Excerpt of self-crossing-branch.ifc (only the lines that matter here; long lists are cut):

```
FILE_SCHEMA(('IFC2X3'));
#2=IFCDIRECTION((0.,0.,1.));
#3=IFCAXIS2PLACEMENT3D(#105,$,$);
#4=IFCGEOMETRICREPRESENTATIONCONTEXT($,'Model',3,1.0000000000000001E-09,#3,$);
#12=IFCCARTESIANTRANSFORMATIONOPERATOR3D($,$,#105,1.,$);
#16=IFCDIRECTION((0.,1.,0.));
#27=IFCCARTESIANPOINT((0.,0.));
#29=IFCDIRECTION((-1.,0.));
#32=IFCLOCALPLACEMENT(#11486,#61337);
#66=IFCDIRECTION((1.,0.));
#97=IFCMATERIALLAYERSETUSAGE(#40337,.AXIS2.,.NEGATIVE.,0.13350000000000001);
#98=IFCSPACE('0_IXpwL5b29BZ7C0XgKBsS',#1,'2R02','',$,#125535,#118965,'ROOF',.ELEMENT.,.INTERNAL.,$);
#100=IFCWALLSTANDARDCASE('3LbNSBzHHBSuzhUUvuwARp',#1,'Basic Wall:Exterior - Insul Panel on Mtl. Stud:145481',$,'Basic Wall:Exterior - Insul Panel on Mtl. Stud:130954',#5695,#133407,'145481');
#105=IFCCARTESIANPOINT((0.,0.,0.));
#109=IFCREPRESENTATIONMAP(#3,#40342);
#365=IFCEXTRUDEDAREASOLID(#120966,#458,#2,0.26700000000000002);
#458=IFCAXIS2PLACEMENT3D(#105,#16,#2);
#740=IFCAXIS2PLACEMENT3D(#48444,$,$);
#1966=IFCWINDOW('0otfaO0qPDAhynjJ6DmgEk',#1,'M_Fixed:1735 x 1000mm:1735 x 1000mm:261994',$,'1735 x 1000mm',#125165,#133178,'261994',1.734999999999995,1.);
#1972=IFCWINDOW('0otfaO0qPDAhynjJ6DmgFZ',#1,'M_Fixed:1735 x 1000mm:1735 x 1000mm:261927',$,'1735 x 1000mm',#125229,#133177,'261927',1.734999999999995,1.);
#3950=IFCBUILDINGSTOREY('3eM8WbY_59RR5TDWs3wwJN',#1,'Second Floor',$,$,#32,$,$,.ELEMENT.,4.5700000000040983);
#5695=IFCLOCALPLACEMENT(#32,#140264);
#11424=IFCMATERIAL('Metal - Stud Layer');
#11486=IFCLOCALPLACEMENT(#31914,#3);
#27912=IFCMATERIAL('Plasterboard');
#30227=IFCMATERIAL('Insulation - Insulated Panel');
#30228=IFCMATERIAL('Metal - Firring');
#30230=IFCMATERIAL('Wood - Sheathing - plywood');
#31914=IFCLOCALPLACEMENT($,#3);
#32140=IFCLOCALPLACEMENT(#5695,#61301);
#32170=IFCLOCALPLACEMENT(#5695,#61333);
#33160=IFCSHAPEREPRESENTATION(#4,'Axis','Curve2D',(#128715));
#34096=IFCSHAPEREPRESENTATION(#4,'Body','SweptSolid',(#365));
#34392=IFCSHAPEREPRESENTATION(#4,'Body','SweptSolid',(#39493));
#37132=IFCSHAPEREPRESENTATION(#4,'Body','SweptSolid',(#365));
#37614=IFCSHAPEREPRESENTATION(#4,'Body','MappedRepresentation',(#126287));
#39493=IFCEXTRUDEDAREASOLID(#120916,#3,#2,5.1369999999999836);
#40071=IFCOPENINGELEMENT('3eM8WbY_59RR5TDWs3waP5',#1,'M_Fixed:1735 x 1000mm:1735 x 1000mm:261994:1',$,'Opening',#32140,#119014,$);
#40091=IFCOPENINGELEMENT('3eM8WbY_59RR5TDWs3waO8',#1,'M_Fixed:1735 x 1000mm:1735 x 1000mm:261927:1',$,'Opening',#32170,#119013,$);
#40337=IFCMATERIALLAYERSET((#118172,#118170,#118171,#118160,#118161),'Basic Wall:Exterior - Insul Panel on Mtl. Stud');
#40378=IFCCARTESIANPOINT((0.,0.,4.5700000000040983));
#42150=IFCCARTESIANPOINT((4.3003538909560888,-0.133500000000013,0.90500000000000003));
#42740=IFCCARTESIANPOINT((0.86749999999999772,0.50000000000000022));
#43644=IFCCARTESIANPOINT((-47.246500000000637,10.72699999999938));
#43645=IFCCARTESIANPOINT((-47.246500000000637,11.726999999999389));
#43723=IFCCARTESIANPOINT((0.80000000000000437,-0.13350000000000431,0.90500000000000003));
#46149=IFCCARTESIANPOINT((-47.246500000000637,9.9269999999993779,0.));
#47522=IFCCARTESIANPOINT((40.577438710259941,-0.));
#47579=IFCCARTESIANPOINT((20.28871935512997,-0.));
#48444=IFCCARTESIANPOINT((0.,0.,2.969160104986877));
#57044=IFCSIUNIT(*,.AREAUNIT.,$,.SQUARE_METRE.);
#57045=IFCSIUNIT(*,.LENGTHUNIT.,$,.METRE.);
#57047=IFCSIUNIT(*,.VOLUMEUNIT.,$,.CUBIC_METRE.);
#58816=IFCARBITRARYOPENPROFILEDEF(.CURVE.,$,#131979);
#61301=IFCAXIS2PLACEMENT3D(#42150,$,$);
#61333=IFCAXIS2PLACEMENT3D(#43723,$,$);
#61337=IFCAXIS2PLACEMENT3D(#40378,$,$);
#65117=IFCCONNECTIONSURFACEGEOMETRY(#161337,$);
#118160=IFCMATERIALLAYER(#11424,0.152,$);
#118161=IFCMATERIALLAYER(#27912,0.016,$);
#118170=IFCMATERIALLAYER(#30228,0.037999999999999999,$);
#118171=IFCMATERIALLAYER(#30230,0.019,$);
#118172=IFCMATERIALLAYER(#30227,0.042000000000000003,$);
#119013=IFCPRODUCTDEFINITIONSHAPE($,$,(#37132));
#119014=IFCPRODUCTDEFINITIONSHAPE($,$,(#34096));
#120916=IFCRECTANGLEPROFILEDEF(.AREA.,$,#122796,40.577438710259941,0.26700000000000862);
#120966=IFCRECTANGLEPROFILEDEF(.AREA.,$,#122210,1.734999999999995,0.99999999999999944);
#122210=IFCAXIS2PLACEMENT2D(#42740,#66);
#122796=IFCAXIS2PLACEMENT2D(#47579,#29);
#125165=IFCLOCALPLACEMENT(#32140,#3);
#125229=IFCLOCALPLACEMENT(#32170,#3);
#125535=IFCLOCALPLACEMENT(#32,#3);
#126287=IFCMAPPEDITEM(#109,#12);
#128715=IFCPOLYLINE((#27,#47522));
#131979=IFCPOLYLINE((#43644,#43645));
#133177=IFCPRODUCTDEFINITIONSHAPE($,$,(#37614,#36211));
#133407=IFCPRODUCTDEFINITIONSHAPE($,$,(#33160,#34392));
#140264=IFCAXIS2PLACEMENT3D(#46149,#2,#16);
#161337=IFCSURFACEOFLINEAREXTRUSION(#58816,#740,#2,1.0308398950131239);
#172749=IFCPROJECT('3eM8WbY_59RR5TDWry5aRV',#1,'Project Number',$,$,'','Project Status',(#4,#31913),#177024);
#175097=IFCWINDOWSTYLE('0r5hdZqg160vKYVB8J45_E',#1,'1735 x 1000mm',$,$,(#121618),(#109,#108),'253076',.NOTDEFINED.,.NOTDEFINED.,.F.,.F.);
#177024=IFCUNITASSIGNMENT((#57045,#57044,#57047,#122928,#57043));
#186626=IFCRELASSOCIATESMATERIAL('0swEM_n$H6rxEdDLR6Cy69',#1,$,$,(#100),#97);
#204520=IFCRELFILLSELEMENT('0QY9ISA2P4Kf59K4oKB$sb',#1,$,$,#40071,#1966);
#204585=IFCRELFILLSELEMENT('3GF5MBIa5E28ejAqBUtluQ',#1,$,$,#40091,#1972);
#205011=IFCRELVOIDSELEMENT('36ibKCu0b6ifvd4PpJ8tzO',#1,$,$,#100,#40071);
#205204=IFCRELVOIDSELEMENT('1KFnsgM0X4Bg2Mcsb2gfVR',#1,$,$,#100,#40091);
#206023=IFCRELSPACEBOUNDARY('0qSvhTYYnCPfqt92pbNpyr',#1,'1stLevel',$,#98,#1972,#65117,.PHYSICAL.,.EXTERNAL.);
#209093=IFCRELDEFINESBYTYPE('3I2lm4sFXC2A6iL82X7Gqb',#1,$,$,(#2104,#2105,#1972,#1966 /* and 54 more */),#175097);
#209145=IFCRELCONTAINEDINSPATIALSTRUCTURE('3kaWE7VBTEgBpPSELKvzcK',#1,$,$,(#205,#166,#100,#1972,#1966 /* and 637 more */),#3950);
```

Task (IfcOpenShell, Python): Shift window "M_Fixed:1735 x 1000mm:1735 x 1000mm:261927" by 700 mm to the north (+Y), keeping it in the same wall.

```python
import numpy as np
import ifcopenshell
import ifcopenshell.api.geometry
import ifcopenshell.util.placement
import ifcopenshell.util.unit

model = ifcopenshell.open("self-crossing-branch.ifc")
unit_scale = ifcopenshell.util.unit.calculate_unit_scale(model)

window = model.by_guid("0otfaO0qPDAhynjJ6DmgFZ")
opening = window.FillsVoids[0].RelatingOpeningElement
wall = opening.VoidsElements[0].RelatingBuildingElement

wall_matrix = ifcopenshell.util.placement.get_local_placement(wall.ObjectPlacement)
shift = wall_matrix[:3, 0] * 0.7 / unit_scale
before = ifcopenshell.util.placement.get_local_placement(window.ObjectPlacement)[:3, 3].copy()

# The window is placed relative to its opening, so it follows when the opening moves.
matrix = ifcopenshell.util.placement.get_local_placement(opening.ObjectPlacement)
matrix[:3, 3] += shift
ifcopenshell.api.geometry.edit_object_placement(
    model, product=opening, matrix=matrix, is_si=False, should_transform_children=True
)

# Space boundary surfaces are stored in each space's coordinates; move them too.
for rel in window.ProvidesBoundaries:
    if not rel.ConnectionGeometry:
        continue
    surface = rel.ConnectionGeometry.SurfaceOnRelatingElement
    space_matrix = ifcopenshell.util.placement.get_local_placement(rel.RelatingSpace.ObjectPlacement)
    point = np.array(surface.Position.Location.Coordinates) + space_matrix[:3, :3].T @ shift
    surface.Position = model.createIfcAxis2Placement3D(
        model.createIfcCartesianPoint(point.tolist()), surface.Position.Axis, surface.Position.RefDirection
    )

after = ifcopenshell.util.placement.get_local_placement(window.ObjectPlacement)[:3, 3]
print("window moved by", (after - before).round(3) + 0.0)

model.write("self-crossing-branch_edited.ifc")
```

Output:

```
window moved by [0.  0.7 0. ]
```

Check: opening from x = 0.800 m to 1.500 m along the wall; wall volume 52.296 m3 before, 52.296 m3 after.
